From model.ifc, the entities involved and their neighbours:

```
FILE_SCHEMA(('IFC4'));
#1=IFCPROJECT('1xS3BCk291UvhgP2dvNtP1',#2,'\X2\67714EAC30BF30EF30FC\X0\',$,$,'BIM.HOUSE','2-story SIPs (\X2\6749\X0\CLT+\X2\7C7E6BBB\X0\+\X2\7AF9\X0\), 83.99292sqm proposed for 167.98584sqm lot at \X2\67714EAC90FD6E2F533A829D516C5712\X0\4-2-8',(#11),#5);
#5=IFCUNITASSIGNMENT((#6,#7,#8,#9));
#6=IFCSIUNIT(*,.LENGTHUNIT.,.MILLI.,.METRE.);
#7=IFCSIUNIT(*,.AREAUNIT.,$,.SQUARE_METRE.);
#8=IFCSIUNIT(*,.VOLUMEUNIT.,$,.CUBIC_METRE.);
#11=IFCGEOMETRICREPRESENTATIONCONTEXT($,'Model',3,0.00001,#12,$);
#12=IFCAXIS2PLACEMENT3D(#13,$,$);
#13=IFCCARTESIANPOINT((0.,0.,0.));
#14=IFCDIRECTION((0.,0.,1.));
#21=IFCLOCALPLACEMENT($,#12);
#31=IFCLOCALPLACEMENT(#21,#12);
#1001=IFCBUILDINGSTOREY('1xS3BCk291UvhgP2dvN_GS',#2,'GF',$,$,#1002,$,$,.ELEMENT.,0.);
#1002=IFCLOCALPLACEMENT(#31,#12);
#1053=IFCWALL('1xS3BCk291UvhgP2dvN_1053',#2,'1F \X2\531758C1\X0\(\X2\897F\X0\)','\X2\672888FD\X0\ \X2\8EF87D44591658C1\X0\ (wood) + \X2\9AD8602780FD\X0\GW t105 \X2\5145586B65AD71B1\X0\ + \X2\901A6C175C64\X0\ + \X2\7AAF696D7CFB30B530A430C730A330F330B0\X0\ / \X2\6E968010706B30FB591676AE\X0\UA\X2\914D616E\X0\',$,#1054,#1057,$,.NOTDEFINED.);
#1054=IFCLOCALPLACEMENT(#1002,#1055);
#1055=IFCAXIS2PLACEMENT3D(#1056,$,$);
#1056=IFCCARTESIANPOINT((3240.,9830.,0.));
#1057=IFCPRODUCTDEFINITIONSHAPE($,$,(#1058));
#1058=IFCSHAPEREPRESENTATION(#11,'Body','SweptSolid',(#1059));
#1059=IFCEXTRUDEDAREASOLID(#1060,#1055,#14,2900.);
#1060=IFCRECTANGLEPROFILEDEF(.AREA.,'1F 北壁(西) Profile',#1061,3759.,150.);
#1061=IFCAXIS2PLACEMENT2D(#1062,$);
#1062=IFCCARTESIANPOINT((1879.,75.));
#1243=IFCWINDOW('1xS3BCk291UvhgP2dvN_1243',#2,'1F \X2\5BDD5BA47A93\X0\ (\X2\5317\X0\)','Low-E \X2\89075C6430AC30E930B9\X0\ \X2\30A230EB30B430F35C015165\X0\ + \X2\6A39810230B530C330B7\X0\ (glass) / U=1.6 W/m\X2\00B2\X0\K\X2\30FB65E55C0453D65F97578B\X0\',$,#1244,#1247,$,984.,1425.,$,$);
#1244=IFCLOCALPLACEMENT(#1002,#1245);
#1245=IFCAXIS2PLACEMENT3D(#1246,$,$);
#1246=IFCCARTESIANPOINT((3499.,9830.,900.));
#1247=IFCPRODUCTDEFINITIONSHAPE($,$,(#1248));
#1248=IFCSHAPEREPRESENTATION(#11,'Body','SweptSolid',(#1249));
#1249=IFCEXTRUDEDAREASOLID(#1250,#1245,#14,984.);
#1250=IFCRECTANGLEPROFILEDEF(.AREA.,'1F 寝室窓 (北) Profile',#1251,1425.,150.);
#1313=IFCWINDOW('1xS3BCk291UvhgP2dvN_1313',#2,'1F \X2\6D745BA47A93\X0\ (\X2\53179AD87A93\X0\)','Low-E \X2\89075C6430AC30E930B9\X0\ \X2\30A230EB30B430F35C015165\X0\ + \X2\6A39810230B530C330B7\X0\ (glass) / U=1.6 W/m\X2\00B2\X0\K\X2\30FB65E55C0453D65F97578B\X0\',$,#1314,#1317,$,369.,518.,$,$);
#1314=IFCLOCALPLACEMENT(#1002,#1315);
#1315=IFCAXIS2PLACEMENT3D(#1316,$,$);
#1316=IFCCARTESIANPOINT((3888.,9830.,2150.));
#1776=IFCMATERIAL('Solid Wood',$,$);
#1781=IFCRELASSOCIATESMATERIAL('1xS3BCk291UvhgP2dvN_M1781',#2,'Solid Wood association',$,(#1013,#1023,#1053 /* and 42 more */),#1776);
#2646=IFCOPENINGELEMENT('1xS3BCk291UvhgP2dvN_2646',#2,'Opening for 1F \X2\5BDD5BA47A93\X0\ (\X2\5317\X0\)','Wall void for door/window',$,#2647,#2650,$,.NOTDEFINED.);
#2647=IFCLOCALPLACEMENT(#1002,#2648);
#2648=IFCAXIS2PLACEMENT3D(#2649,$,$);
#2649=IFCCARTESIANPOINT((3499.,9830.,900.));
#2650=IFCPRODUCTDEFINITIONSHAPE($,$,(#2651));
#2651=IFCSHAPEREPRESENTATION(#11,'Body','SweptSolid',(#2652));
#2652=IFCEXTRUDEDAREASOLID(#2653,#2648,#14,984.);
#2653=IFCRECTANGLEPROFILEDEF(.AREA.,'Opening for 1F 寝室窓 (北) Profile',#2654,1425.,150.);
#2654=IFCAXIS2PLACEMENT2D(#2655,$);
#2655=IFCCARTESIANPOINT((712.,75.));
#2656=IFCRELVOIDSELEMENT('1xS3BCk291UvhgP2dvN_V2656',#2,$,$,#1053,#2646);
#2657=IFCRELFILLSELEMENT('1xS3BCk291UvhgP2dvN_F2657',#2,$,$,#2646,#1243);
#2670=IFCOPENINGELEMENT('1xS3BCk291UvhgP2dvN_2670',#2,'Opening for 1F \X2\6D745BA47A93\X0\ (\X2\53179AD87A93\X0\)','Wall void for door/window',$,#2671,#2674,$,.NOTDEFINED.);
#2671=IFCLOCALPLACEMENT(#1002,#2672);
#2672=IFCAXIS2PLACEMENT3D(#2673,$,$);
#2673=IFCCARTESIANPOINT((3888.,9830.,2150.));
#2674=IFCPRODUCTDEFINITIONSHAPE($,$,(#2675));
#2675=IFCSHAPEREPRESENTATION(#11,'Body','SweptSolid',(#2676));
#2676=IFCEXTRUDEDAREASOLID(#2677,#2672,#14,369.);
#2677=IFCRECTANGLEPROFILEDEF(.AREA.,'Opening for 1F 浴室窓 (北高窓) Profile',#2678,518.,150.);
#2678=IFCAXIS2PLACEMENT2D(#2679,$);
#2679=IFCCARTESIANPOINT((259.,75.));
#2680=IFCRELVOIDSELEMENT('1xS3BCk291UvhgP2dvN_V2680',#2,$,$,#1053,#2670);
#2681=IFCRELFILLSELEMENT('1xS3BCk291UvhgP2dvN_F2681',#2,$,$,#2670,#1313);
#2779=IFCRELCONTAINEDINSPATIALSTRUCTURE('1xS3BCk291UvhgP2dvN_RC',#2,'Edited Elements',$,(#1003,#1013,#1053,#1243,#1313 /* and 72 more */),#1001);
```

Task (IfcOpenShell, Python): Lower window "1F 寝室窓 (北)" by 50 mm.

```python
import numpy as np
import ifcopenshell
import ifcopenshell.api.geometry
import ifcopenshell.util.placement
import ifcopenshell.util.unit

model = ifcopenshell.open("model.ifc")
unit_scale = ifcopenshell.util.unit.calculate_unit_scale(model)

window = model.by_guid("1xS3BCk291UvhgP2dvN_1243")
opening = window.FillsVoids[0].RelatingOpeningElement
dz = -0.05 / unit_scale

shift = np.array([0.0, 0.0, dz])
# The window is not placed relative to its opening, so move both.
for product in (opening, window):
    matrix = ifcopenshell.util.placement.get_local_placement(product.ObjectPlacement)
    matrix[:3, 3] += shift
    ifcopenshell.api.geometry.edit_object_placement(model, product=product, matrix=matrix, is_si=False)

print(f"moved by {dz * unit_scale:+.3f} m")

model.write("model_edited.ifc")
```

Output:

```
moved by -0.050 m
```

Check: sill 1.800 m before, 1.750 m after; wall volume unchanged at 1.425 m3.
